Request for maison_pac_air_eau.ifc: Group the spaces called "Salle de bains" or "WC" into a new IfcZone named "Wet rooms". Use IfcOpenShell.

First a look at what the model holds.

```python
import ifcopenshell

model = ifcopenshell.open("maison_pac_air_eau.ifc")
print(model.schema)
seen = {}
for space in model.by_type("IfcSpace"):
    seen[space.LongName] = seen.get(space.LongName, 0) + 1
for name, count in sorted(seen.items(), key=str):
    print(count, "x", name)
print("zones:", [z.Name for z in model.by_type("IfcZone")][:20])
```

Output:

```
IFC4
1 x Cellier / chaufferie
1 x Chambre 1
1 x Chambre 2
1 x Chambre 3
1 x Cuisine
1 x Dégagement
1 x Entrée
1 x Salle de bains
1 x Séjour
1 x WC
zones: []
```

```python
import ifcopenshell
import ifcopenshell.api.group
import ifcopenshell.api.root

model = ifcopenshell.open("maison_pac_air_eau.ifc")

names = {"Salle de bains", "WC"}
spaces = [s for s in model.by_type("IfcSpace") if s.LongName in names]

zone = ifcopenshell.api.root.create_entity(model, ifc_class="IfcZone", name="Wet rooms")
ifcopenshell.api.group.assign_group(model, products=spaces, group=zone)
print(len(spaces), "spaces in", zone.Name)

model.write("maison_pac_air_eau_edited.ifc")
```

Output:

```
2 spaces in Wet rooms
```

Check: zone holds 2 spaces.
